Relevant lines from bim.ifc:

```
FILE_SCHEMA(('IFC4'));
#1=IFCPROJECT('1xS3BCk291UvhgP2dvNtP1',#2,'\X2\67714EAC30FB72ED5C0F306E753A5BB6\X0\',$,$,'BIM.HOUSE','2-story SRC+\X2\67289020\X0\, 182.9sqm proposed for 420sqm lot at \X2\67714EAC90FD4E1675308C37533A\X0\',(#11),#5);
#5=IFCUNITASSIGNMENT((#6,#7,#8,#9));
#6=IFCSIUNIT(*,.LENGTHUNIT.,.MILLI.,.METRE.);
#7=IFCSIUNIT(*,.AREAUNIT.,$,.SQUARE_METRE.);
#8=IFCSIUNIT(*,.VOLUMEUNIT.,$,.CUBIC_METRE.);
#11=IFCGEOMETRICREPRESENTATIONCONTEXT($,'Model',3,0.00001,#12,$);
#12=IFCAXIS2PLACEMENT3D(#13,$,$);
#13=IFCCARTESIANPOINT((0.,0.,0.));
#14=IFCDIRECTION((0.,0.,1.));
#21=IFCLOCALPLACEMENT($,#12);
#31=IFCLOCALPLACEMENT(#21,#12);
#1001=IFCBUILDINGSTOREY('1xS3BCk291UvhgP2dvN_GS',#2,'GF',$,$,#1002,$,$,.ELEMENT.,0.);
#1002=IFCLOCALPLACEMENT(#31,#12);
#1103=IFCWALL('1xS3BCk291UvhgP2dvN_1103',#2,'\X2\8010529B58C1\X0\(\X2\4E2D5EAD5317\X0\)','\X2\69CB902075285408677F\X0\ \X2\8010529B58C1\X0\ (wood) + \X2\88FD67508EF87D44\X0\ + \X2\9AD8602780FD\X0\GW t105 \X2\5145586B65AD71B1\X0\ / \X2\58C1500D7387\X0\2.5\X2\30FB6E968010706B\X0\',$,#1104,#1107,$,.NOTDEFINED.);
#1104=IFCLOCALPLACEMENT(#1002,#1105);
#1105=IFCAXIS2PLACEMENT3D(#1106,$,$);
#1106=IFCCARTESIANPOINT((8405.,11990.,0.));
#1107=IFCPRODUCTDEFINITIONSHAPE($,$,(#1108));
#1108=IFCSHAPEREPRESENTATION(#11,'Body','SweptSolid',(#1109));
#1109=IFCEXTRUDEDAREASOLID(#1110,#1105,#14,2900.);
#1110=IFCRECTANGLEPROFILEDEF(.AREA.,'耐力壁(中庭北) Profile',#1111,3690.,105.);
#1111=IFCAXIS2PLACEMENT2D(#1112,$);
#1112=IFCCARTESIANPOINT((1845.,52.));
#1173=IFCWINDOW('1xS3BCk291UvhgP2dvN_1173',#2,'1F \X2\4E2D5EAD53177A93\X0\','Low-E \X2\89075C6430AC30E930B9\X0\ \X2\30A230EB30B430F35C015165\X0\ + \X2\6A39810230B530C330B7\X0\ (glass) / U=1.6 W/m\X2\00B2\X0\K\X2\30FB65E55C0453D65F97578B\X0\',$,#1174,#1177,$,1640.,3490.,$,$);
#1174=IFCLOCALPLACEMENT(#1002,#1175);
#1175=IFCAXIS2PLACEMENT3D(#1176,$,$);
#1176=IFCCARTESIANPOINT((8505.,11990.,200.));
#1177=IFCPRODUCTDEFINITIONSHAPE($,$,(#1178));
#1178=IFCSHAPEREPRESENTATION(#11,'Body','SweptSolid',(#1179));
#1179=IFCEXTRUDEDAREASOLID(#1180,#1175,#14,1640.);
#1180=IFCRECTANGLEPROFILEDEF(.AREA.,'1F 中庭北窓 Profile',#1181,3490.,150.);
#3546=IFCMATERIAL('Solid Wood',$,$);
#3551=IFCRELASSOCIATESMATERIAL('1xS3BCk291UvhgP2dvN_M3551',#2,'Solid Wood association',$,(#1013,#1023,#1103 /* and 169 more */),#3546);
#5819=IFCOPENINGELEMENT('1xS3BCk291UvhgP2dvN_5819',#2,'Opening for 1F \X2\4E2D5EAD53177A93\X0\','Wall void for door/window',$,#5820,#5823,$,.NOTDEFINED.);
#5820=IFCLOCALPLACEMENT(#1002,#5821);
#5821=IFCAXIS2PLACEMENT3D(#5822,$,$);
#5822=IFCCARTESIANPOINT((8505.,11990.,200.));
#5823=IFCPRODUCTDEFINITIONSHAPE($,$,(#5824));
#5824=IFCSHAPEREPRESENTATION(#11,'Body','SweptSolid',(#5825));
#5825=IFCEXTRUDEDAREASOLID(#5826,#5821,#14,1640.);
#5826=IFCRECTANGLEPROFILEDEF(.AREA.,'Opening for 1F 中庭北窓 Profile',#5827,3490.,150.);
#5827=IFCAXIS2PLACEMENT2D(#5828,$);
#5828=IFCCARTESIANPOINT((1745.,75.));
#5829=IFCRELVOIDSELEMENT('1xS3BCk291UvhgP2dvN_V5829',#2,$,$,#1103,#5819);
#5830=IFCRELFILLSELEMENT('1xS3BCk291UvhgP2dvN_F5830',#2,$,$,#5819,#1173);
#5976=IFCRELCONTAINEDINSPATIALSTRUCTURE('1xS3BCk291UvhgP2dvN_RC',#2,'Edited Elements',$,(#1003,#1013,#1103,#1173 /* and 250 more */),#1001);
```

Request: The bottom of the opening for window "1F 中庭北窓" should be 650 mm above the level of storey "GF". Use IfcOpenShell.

```python
import numpy as np
import ifcopenshell
import ifcopenshell.api.geometry
import ifcopenshell.geom
import ifcopenshell.util.element
import ifcopenshell.util.placement
import ifcopenshell.util.shape
import ifcopenshell.util.unit

model = ifcopenshell.open("bim.ifc")
unit_scale = ifcopenshell.util.unit.calculate_unit_scale(model)

window = model.by_guid("1xS3BCk291UvhgP2dvN_1173")
opening = window.FillsVoids[0].RelatingOpeningElement
storey = ifcopenshell.util.element.get_container(window, ifc_class="IfcBuildingStorey")
level = ifcopenshell.util.placement.get_local_placement(storey.ObjectPlacement)[2, 3]

# The opening's origin need not be at the sill, so measure its lowest point.
shape = ifcopenshell.geom.create_shape(ifcopenshell.geom.settings(), opening)
bottom = ifcopenshell.util.shape.get_shape_bottom_elevation(shape, shape.geometry) / unit_scale
dz = level + 650.0 - bottom

shift = np.array([0.0, 0.0, dz])
# The window is not placed relative to its opening, so move both.
for product in (opening, window):
    matrix = ifcopenshell.util.placement.get_local_placement(product.ObjectPlacement)
    matrix[:3, 3] += shift
    ifcopenshell.api.geometry.edit_object_placement(model, product=product, matrix=matrix, is_si=False)

print(f"moved by {dz * unit_scale:+.3f} m")

model.write("bim_updated.ifc")
```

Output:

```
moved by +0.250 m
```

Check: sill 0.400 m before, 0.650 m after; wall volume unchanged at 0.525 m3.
